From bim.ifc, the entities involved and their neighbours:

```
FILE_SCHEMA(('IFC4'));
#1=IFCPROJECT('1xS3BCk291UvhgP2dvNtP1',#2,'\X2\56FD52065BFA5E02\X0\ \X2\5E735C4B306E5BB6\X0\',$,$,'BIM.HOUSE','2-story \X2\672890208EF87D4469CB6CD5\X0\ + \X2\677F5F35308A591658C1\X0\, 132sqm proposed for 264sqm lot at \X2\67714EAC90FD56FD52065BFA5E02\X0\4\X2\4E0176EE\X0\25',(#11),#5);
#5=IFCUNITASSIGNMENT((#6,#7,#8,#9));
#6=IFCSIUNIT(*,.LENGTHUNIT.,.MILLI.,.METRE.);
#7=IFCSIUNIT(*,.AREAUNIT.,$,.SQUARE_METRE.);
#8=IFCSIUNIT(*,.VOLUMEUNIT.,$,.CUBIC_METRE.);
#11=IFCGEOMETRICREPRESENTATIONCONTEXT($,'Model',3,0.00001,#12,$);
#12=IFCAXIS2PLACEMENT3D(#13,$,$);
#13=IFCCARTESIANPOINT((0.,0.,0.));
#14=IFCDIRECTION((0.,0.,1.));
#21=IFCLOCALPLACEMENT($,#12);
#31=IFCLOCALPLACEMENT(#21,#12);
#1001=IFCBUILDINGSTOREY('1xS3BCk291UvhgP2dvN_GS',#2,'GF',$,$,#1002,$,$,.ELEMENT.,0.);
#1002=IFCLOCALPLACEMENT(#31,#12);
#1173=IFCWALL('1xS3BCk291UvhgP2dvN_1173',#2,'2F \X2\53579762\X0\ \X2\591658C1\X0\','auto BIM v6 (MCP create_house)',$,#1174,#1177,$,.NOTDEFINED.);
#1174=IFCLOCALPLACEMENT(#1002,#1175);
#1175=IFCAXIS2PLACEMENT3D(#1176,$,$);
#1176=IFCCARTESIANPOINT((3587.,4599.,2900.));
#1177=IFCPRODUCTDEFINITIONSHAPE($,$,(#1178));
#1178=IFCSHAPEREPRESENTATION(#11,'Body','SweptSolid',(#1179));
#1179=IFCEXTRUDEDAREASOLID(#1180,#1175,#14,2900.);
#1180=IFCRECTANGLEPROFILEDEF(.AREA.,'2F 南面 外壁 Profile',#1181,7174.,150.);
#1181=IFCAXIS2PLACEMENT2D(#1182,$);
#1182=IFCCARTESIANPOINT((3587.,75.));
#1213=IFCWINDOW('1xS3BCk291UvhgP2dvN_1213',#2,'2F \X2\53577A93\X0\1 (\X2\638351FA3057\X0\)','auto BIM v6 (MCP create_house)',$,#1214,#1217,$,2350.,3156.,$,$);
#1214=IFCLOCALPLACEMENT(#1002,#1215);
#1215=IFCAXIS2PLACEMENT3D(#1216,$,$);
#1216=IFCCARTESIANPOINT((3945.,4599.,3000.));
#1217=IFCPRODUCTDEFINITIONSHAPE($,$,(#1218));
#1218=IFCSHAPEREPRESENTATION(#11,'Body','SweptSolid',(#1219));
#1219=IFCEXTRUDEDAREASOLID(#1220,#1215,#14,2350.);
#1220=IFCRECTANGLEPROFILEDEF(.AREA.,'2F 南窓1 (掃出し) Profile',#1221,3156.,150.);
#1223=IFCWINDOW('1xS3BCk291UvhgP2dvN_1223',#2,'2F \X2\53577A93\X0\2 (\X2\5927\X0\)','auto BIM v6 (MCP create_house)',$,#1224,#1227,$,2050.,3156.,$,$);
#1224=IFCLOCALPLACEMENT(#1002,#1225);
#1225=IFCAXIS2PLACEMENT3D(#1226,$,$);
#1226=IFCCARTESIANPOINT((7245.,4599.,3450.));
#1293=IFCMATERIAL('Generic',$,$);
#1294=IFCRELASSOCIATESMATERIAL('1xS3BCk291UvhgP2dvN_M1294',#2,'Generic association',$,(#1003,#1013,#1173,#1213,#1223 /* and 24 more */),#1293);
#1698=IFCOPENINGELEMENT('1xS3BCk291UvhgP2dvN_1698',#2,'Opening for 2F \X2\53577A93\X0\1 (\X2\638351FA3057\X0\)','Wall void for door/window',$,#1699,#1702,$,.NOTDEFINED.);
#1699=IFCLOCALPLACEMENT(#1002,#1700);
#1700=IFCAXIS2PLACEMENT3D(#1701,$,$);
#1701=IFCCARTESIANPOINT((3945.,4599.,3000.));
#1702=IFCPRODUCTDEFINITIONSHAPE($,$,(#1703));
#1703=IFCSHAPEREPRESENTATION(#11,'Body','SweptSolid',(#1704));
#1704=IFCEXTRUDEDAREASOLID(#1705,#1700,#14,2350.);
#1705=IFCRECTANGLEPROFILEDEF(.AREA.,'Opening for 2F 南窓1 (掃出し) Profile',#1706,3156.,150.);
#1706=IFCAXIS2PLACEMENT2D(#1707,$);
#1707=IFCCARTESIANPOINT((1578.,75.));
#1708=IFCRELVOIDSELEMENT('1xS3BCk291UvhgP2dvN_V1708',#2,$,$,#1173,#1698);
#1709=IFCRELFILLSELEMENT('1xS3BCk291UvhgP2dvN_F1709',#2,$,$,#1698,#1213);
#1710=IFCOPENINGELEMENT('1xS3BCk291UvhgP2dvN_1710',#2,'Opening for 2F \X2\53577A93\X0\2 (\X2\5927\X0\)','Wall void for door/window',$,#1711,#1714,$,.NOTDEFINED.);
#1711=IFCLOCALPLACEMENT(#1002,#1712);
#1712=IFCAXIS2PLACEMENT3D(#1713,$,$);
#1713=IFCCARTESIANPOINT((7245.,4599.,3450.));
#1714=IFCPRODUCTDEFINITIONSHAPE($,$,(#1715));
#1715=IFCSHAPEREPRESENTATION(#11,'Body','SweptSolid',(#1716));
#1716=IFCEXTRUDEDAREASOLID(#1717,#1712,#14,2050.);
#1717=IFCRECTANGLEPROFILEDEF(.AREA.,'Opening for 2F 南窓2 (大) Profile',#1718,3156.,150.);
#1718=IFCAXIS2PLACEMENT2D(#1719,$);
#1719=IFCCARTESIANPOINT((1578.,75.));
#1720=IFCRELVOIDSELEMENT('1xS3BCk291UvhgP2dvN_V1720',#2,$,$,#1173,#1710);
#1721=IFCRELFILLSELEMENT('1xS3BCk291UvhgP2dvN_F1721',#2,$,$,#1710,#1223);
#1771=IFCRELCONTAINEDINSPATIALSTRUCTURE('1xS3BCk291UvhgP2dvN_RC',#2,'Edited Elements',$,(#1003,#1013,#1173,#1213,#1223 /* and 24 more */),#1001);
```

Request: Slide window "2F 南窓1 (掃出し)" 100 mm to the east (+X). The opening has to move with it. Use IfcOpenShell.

```python
import ifcopenshell
import ifcopenshell.api.geometry
import ifcopenshell.util.placement
import ifcopenshell.util.unit

model = ifcopenshell.open("bim.ifc")
unit_scale = ifcopenshell.util.unit.calculate_unit_scale(model)

window = model.by_id(1213)
opening = window.FillsVoids[0].RelatingOpeningElement
wall = opening.VoidsElements[0].RelatingBuildingElement

wall_matrix = ifcopenshell.util.placement.get_local_placement(wall.ObjectPlacement)
shift = wall_matrix[:3, 0] * 0.1 / unit_scale
before = ifcopenshell.util.placement.get_local_placement(window.ObjectPlacement)[:3, 3].copy()

# The window is not placed relative to its opening, so move both.
for product in (opening, window):
    matrix = ifcopenshell.util.placement.get_local_placement(product.ObjectPlacement)
    matrix[:3, 3] += shift
    ifcopenshell.api.geometry.edit_object_placement(model, product=product, matrix=matrix, is_si=False)

after = ifcopenshell.util.placement.get_local_placement(window.ObjectPlacement)[:3, 3]
print("window moved by", (after - before).round(3) + 0.0)

model.write("bim_rev.ifc")
```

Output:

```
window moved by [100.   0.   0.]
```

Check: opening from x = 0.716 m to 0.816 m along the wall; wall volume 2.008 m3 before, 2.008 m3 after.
